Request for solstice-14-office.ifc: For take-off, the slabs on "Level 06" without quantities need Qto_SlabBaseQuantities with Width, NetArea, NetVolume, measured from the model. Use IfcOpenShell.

First a look at what the model holds.

```python
import ifcopenshell
import ifcopenshell.util.element
import ifcopenshell.util.unit

model = ifcopenshell.open("solstice-14-office.ifc")
print(model.schema)
for unit_type in ("LENGTHUNIT", "AREAUNIT", "VOLUMEUNIT"):
    print(unit_type, ifcopenshell.util.unit.calculate_unit_scale(model, unit_type))
storey = next(s for s in model.by_type("IfcBuildingStorey") if s.Name == "Level 06")
slabs = [e for e in ifcopenshell.util.element.get_decomposition(storey) if e.is_a("IfcSlab")]
for e in sorted(slabs, key=lambda e: e.id()):
    print(e.id(), e.is_a(), e.Name, list(ifcopenshell.util.element.get_psets(e, qtos_only=True)), sep=" | ")
```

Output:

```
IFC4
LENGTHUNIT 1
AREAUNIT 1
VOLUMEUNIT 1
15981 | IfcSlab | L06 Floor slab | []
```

```python
import ifcopenshell
import ifcopenshell.api.pset
import ifcopenshell.geom
import ifcopenshell.util.element
import ifcopenshell.util.shape
import ifcopenshell.util.unit

model = ifcopenshell.open("solstice-14-office.ifc")
unit_scale = ifcopenshell.util.unit.calculate_unit_scale(model)
area_scale = ifcopenshell.util.unit.calculate_unit_scale(model, "AREAUNIT")
volume_scale = ifcopenshell.util.unit.calculate_unit_scale(model, "VOLUMEUNIT")
settings = ifcopenshell.geom.settings()

storey = next(s for s in model.by_type("IfcBuildingStorey") if s.Name == "Level 06")
slabs = [e for e in ifcopenshell.util.element.get_decomposition(storey) if e.is_a("IfcSlab")]

for e in sorted(slabs, key=lambda e: e.id()):
    if ifcopenshell.util.element.get_psets(e, qtos_only=True, should_inherit=False):
        continue
    # Geometry comes back in metres, in the element's own axes.
    shape = ifcopenshell.geom.create_shape(settings, e)
    values = {
        "Width": ifcopenshell.util.shape.get_z(shape.geometry) / unit_scale,
        "NetArea": ifcopenshell.util.shape.get_footprint_area(shape.geometry) / area_scale,
        "NetVolume": ifcopenshell.util.shape.get_volume(shape.geometry) / volume_scale,
    }
    qto = ifcopenshell.api.pset.add_qto(model, product=e, name="Qto_SlabBaseQuantities")
    ifcopenshell.api.pset.edit_qto(model, qto=qto, properties=values)
    print(e.id(), {k: round(v, 3) for k, v in values.items()})

model.write("solstice-14-office-out.ifc")
```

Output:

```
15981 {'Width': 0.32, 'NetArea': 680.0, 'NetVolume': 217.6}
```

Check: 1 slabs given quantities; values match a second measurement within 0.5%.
